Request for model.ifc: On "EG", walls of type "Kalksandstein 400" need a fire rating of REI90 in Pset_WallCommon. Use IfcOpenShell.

First a look at what the model holds.

```python
import ifcopenshell
import ifcopenshell.util.element

model = ifcopenshell.open("model.ifc")
print(model.schema)
storey = next(s for s in model.by_type("IfcBuildingStorey") if s.Name == "EG")
walls = [e for e in ifcopenshell.util.element.get_decomposition(storey) if e.is_a("IfcWall")]
seen = {}
for e in walls:
    element_type = ifcopenshell.util.element.get_type(e)
    key = (element_type.Name if element_type != e and element_type else None, ifcopenshell.util.element.get_pset(e, "Pset_WallCommon", "FireRating"))
    seen[key] = seen.get(key, 0) + 1
for (name, value), count in sorted(seen.items(), key=str):
    print(count, "x", name, "|", value)
```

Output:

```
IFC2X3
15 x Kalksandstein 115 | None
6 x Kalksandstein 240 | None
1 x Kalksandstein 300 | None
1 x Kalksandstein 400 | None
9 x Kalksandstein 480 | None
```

```python
import ifcopenshell
import ifcopenshell.api.pset
import ifcopenshell.util.element

model = ifcopenshell.open("model.ifc")

storey = next(s for s in model.by_type("IfcBuildingStorey") if s.Name == "EG")
walls = [e for e in ifcopenshell.util.element.get_decomposition(storey) if e.is_a("IfcWall")]

count = 0
for e in walls:
    element_type = ifcopenshell.util.element.get_type(e)
    if element_type in (None, e) or element_type.Name != "Kalksandstein 400":
        continue
    # add_pset returns the element's existing set when there is one.
    pset = ifcopenshell.api.pset.add_pset(model, product=e, name="Pset_WallCommon")
    ifcopenshell.api.pset.edit_pset(model, pset=pset, properties={"FireRating": "REI90"})
    count += 1

print(count, "walls updated")

model.write("model_v2.ifc")
```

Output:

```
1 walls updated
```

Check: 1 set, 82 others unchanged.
